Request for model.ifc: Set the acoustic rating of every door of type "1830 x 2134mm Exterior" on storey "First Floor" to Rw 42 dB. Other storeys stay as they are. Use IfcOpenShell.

First a look at what the model holds.

```python
import ifcopenshell
import ifcopenshell.util.element

model = ifcopenshell.open("model.ifc")
print(model.schema)
storey = next(s for s in model.by_type("IfcBuildingStorey") if s.Name == "First Floor")
doors = [e for e in ifcopenshell.util.element.get_decomposition(storey) if e.is_a("IfcDoor")]
seen = {}
for e in doors:
    element_type = ifcopenshell.util.element.get_type(e)
    key = (element_type.Name if element_type != e and element_type else None, ifcopenshell.util.element.get_pset(e, "Pset_DoorCommon", "AcousticRating"))
    seen[key] = seen.get(key, 0) + 1
for (name, value), count in sorted(seen.items(), key=str):
    print(count, "x", name, "|", value)
```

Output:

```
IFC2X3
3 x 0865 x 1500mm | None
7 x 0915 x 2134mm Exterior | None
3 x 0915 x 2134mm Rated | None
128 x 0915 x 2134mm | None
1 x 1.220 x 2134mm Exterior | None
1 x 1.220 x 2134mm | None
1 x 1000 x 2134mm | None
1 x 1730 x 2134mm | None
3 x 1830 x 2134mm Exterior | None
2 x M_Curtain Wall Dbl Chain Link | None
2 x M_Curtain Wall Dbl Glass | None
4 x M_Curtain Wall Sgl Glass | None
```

```python
import ifcopenshell
import ifcopenshell.api.pset
import ifcopenshell.util.element

model = ifcopenshell.open("model.ifc")

storey = next(s for s in model.by_type("IfcBuildingStorey") if s.Name == "First Floor")
doors = [e for e in ifcopenshell.util.element.get_decomposition(storey) if e.is_a("IfcDoor")]

count = 0
for e in doors:
    element_type = ifcopenshell.util.element.get_type(e)
    if element_type in (None, e) or element_type.Name != "1830 x 2134mm Exterior":
        continue
    # add_pset returns the element's existing set when there is one.
    pset = ifcopenshell.api.pset.add_pset(model, product=e, name="Pset_DoorCommon")
    ifcopenshell.api.pset.edit_pset(model, pset=pset, properties={"AcousticRating": "Rw 42 dB"})
    count += 1

print(count, "doors updated")

model.write("model_updated.ifc")
```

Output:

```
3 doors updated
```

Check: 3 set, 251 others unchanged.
